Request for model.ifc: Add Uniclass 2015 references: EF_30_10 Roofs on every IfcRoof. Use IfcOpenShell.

First a look at what the model holds.

```python
import ifcopenshell

model = ifcopenshell.open("model.ifc")
print(model.schema)
print("classifications:", [c.Name for c in model.by_type("IfcClassification")])
for ifc_class in ("IfcDoor", "IfcRoof", "IfcStair", "IfcWall", "IfcWindow"):
    print(ifc_class, len(model.by_type(ifc_class)))
```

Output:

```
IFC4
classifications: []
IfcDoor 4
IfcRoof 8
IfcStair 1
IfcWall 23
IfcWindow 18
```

```python
import ifcopenshell
import ifcopenshell.api.classification

model = ifcopenshell.open("model.ifc")

system = ifcopenshell.api.classification.add_classification(model, classification="Uniclass 2015")

codes = {
    "IfcRoof": ("EF_30_10", "Roofs"),
}
for ifc_class, (code, name) in codes.items():
    products = model.by_type(ifc_class)
    ifcopenshell.api.classification.add_reference(
        model, products=products, classification=system, identification=code, name=name
    )
    print(code, len(products))

model.write("model_updated.ifc")
```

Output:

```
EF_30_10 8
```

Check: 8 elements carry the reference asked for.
